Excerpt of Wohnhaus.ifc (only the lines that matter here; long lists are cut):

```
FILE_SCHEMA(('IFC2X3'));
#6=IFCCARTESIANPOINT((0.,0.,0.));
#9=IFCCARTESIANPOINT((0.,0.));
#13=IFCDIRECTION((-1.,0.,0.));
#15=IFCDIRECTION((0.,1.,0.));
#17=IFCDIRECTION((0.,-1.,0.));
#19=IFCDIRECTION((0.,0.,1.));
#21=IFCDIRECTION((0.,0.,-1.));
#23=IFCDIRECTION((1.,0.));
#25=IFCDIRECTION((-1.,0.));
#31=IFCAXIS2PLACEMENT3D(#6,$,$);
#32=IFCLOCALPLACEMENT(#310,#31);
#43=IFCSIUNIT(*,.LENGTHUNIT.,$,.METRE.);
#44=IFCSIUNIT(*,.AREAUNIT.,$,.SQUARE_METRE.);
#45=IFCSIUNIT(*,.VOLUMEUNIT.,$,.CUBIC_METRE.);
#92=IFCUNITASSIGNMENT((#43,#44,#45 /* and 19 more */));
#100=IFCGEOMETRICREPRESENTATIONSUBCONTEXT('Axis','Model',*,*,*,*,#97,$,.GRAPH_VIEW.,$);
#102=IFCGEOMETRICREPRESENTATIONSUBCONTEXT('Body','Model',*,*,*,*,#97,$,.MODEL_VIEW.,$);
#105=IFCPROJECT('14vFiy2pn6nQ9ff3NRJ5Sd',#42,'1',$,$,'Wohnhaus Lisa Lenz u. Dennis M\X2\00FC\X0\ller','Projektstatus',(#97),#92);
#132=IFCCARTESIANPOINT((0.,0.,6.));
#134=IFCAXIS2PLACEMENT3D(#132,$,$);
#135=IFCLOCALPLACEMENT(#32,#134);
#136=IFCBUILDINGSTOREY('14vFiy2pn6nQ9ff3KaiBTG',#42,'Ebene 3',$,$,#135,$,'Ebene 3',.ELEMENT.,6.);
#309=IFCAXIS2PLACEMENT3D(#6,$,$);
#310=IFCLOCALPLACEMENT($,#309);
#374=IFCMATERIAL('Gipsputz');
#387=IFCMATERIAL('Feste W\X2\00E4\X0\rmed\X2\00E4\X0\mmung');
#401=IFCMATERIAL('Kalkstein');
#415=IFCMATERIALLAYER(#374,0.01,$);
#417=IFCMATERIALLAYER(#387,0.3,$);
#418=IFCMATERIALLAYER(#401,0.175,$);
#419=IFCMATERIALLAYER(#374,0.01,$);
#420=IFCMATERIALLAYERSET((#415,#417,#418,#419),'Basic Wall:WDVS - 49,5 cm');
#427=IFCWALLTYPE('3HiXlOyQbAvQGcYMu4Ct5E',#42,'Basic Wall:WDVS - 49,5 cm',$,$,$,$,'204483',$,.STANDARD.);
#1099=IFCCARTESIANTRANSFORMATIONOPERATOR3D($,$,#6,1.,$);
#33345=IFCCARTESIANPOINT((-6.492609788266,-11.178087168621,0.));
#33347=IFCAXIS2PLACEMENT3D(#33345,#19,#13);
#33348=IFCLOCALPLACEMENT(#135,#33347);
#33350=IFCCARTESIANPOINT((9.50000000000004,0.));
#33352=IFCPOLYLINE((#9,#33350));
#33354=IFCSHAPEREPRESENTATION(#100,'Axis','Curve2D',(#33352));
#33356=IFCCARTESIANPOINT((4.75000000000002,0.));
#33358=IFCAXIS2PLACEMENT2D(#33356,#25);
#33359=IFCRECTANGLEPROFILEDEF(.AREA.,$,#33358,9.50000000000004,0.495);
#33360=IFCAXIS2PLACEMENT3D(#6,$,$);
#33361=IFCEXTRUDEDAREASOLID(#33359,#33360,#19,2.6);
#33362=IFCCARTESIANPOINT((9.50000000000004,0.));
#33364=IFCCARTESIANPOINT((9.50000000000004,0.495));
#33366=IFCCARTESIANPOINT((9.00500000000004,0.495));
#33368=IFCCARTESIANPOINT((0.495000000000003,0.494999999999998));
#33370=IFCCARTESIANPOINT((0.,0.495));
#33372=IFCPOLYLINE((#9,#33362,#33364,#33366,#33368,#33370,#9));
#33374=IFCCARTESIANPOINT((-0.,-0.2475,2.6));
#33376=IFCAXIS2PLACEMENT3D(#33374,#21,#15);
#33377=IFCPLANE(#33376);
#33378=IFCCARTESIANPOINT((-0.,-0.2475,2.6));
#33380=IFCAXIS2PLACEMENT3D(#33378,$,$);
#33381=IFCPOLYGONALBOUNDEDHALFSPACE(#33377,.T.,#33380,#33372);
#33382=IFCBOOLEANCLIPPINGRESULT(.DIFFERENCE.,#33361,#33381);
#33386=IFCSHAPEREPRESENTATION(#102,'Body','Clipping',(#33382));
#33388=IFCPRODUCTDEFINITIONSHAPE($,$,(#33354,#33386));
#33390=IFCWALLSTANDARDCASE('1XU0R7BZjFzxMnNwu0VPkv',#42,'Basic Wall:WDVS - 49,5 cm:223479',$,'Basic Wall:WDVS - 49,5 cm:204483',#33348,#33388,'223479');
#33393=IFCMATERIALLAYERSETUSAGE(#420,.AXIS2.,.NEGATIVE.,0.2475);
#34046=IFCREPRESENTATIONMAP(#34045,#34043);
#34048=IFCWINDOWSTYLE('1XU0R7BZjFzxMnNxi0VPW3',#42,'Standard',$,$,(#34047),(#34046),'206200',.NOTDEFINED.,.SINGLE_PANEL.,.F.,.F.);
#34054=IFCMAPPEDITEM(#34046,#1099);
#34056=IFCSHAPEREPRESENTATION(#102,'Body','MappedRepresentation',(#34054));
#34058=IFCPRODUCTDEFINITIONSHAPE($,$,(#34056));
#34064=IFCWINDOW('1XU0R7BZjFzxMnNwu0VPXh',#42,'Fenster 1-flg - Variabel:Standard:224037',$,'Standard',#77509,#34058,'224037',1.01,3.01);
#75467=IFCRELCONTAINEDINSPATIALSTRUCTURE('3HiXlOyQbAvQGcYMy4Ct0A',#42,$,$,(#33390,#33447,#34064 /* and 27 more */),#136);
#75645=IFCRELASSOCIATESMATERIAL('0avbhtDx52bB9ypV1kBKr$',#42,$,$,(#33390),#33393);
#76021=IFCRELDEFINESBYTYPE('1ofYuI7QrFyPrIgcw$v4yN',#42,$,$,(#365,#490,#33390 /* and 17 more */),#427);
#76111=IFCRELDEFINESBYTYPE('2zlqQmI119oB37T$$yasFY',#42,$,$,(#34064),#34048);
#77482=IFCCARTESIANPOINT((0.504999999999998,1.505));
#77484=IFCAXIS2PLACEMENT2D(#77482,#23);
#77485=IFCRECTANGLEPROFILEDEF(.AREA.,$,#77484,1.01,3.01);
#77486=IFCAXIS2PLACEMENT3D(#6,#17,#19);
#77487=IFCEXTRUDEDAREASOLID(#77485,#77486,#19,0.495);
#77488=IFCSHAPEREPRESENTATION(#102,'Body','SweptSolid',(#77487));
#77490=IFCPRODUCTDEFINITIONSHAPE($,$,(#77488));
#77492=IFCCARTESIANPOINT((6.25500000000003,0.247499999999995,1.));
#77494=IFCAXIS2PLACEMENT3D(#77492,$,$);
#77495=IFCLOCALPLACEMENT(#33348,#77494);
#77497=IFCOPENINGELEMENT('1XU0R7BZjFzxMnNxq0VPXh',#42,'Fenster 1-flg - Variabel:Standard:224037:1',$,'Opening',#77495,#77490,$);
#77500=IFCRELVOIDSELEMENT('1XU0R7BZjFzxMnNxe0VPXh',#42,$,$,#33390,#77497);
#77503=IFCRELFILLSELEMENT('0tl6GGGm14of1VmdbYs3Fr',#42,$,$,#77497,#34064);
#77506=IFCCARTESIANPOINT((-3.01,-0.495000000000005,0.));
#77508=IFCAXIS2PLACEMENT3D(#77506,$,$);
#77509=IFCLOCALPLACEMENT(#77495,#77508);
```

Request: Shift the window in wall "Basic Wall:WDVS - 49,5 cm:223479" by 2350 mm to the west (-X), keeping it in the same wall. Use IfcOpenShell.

```python
import ifcopenshell
import ifcopenshell.api.geometry
import ifcopenshell.util.placement
import ifcopenshell.util.unit

model = ifcopenshell.open("Wohnhaus.ifc")
unit_scale = ifcopenshell.util.unit.calculate_unit_scale(model)

window = model.by_guid("1XU0R7BZjFzxMnNwu0VPXh")
opening = window.FillsVoids[0].RelatingOpeningElement
wall = opening.VoidsElements[0].RelatingBuildingElement

wall_matrix = ifcopenshell.util.placement.get_local_placement(wall.ObjectPlacement)
shift = wall_matrix[:3, 0] * 2.35 / unit_scale
before = ifcopenshell.util.placement.get_local_placement(window.ObjectPlacement)[:3, 3].copy()

# The window is placed relative to its opening, so it follows when the opening moves.
matrix = ifcopenshell.util.placement.get_local_placement(opening.ObjectPlacement)
matrix[:3, 3] += shift
ifcopenshell.api.geometry.edit_object_placement(
    model, product=opening, matrix=matrix, is_si=False, should_transform_children=True
)

after = ifcopenshell.util.placement.get_local_placement(window.ObjectPlacement)[:3, 3]
print("window moved by", (after - before).round(3) + 0.0)

model.write("Wohnhaus_rev.ifc")
```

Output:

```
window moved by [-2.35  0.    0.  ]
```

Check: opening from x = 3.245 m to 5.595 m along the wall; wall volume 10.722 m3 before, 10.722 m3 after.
